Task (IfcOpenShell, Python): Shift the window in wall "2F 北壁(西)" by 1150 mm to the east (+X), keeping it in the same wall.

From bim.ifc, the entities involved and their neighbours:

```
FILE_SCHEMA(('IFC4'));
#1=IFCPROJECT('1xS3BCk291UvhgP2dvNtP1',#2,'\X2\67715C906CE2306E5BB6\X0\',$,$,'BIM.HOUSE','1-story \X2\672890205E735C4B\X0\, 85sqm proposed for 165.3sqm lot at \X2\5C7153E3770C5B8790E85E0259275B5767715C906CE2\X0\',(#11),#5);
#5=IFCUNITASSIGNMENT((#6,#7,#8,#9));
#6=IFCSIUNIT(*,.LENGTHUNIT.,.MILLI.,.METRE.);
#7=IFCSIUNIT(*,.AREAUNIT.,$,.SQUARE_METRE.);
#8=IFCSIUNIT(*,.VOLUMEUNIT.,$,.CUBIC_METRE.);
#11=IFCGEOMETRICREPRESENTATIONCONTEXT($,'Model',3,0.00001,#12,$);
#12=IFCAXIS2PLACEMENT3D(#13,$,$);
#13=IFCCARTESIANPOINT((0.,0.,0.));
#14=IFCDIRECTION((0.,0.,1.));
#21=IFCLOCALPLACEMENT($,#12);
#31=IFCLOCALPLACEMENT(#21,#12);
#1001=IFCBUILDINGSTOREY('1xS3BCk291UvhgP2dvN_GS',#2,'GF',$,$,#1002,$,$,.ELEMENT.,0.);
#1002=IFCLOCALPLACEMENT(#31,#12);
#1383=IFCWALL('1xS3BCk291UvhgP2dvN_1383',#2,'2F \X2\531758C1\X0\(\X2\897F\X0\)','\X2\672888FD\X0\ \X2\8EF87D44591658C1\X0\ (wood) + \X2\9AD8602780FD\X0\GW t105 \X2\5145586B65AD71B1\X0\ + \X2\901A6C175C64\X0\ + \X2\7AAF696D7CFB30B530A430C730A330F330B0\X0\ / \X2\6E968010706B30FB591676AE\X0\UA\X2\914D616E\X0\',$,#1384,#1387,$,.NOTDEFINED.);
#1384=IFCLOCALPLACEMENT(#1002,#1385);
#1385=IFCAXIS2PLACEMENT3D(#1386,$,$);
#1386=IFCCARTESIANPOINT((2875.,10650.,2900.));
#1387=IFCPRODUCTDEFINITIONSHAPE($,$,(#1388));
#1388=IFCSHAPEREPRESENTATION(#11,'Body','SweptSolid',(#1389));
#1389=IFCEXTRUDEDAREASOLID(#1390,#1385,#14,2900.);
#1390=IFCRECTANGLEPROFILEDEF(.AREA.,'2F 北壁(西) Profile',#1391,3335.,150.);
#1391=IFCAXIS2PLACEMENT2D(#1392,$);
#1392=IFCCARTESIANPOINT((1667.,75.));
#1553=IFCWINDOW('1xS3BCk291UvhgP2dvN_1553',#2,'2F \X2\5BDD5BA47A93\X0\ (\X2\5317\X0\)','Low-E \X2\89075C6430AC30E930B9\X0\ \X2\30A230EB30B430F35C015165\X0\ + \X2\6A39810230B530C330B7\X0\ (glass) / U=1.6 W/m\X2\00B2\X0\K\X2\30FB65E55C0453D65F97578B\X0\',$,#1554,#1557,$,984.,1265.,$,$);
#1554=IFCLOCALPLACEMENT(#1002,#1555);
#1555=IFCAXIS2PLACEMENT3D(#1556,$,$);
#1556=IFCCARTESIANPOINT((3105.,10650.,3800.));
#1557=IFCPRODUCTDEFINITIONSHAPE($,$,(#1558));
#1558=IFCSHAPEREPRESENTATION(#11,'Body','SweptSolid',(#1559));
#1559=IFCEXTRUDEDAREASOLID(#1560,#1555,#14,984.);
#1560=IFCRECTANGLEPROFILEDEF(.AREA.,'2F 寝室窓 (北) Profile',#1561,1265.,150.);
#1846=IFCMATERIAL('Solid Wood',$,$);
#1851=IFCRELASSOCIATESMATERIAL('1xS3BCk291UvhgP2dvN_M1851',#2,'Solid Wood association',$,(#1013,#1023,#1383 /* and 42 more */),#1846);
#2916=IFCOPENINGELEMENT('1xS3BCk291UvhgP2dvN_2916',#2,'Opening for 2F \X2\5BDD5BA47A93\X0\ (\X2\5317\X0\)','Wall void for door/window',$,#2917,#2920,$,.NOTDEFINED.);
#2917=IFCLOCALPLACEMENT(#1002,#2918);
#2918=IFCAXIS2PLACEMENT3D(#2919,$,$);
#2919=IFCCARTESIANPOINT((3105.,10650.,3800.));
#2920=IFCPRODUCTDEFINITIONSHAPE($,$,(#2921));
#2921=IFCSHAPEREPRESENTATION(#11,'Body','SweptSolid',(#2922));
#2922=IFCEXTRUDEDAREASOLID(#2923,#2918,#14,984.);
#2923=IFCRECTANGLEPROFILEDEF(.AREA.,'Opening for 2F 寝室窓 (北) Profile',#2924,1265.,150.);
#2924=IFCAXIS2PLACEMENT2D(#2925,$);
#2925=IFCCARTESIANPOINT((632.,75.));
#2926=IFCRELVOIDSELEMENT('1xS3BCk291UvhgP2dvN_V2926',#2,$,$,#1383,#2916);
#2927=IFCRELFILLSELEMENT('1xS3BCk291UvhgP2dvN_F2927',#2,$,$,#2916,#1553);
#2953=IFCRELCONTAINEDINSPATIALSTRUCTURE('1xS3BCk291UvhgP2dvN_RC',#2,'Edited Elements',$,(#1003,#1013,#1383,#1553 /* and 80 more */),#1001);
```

```python
import ifcopenshell
import ifcopenshell.api.geometry
import ifcopenshell.util.placement
import ifcopenshell.util.unit

model = ifcopenshell.open("bim.ifc")
unit_scale = ifcopenshell.util.unit.calculate_unit_scale(model)

window = model.by_guid("1xS3BCk291UvhgP2dvN_1553")
opening = window.FillsVoids[0].RelatingOpeningElement
wall = opening.VoidsElements[0].RelatingBuildingElement

wall_matrix = ifcopenshell.util.placement.get_local_placement(wall.ObjectPlacement)
shift = wall_matrix[:3, 0] * 1.15 / unit_scale
before = ifcopenshell.util.placement.get_local_placement(window.ObjectPlacement)[:3, 3].copy()

# The window is not placed relative to its opening, so move both.
for product in (opening, window):
    matrix = ifcopenshell.util.placement.get_local_placement(product.ObjectPlacement)
    matrix[:3, 3] += shift
    ifcopenshell.api.geometry.edit_object_placement(model, product=product, matrix=matrix, is_si=False)

after = ifcopenshell.util.placement.get_local_placement(window.ObjectPlacement)[:3, 3]
print("window moved by", (after - before).round(3) + 0.0)

model.write("bim_rev.ifc")
```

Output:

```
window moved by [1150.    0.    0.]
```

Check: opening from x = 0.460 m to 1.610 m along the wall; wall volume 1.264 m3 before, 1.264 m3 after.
